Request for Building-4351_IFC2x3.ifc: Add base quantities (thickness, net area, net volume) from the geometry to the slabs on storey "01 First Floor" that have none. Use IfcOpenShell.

First a look at what the model holds.

```python
import ifcopenshell
import ifcopenshell.util.element
import ifcopenshell.util.unit

model = ifcopenshell.open("Building-4351_IFC2x3.ifc")
print(model.schema)
for unit_type in ("LENGTHUNIT", "AREAUNIT", "VOLUMEUNIT"):
    print(unit_type, ifcopenshell.util.unit.calculate_unit_scale(model, unit_type))
storey = next(s for s in model.by_type("IfcBuildingStorey") if s.Name == "01 First Floor")
slabs = [e for e in ifcopenshell.util.element.get_decomposition(storey) if e.is_a("IfcSlab")]
for e in sorted(slabs, key=lambda e: e.id()):
    print(e.id(), e.is_a(), e.Name, list(ifcopenshell.util.element.get_psets(e, qtos_only=True)), sep=" | ")
```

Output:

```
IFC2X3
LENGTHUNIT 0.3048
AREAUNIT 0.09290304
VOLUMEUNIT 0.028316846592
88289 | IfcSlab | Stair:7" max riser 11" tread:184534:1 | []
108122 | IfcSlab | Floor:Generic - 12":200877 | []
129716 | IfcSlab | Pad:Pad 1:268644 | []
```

```python
import ifcopenshell
import ifcopenshell.api.pset
import ifcopenshell.geom
import ifcopenshell.util.element
import ifcopenshell.util.shape
import ifcopenshell.util.unit

model = ifcopenshell.open("Building-4351_IFC2x3.ifc")
unit_scale = ifcopenshell.util.unit.calculate_unit_scale(model)
area_scale = ifcopenshell.util.unit.calculate_unit_scale(model, "AREAUNIT")
volume_scale = ifcopenshell.util.unit.calculate_unit_scale(model, "VOLUMEUNIT")
settings = ifcopenshell.geom.settings()

storey = next(s for s in model.by_type("IfcBuildingStorey") if s.Name == "01 First Floor")
slabs = [e for e in ifcopenshell.util.element.get_decomposition(storey) if e.is_a("IfcSlab")]

for e in sorted(slabs, key=lambda e: e.id()):
    if ifcopenshell.util.element.get_psets(e, qtos_only=True, should_inherit=False):
        continue
    # Geometry comes back in metres, in the element's own axes.
    shape = ifcopenshell.geom.create_shape(settings, e)
    values = {
        "Width": ifcopenshell.util.shape.get_z(shape.geometry) / unit_scale,
        "NetArea": ifcopenshell.util.shape.get_footprint_area(shape.geometry) / area_scale,
        "NetVolume": ifcopenshell.util.shape.get_volume(shape.geometry) / volume_scale,
    }
    qto = ifcopenshell.api.pset.add_qto(model, product=e, name="BaseQuantities")
    ifcopenshell.api.pset.edit_qto(model, qto=qto, properties=values)
    print(e.id(), {k: round(v, 3) for k, v in values.items()})

model.write("Building-4351_IFC2x3_rev.ifc")
```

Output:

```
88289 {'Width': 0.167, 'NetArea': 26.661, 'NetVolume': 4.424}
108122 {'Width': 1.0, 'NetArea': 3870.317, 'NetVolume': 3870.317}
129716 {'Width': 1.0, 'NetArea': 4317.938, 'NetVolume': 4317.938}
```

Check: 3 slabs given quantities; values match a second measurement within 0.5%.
